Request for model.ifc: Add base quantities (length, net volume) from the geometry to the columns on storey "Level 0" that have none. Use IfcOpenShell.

First a look at what the model holds.

```python
import ifcopenshell
import ifcopenshell.util.element
import ifcopenshell.util.unit

model = ifcopenshell.open("model.ifc")
print(model.schema)
for unit_type in ("LENGTHUNIT", "AREAUNIT", "VOLUMEUNIT"):
    print(unit_type, ifcopenshell.util.unit.calculate_unit_scale(model, unit_type))
storey = next(s for s in model.by_type("IfcBuildingStorey") if s.Name == "Level 0")
columns = [e for e in ifcopenshell.util.element.get_decomposition(storey) if e.is_a("IfcColumn")]
for e in sorted(columns, key=lambda e: e.id()):
    print(e.id(), e.is_a(), e.Name, list(ifcopenshell.util.element.get_psets(e, qtos_only=True)), sep=" | ")
```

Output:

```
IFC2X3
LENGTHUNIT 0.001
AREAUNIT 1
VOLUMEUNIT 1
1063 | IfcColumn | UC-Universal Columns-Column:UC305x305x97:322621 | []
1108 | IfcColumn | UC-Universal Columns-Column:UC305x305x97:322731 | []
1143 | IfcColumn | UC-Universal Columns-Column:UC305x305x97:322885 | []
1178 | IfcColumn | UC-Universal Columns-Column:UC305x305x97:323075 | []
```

```python
import ifcopenshell
import ifcopenshell.api.pset
import ifcopenshell.geom
import ifcopenshell.util.element
import ifcopenshell.util.shape
import ifcopenshell.util.unit

model = ifcopenshell.open("model.ifc")
unit_scale = ifcopenshell.util.unit.calculate_unit_scale(model)
volume_scale = ifcopenshell.util.unit.calculate_unit_scale(model, "VOLUMEUNIT")
settings = ifcopenshell.geom.settings()

storey = next(s for s in model.by_type("IfcBuildingStorey") if s.Name == "Level 0")
columns = [e for e in ifcopenshell.util.element.get_decomposition(storey) if e.is_a("IfcColumn")]

for e in sorted(columns, key=lambda e: e.id()):
    if ifcopenshell.util.element.get_psets(e, qtos_only=True, should_inherit=False):
        continue
    # Geometry comes back in metres, in the element's own axes.
    shape = ifcopenshell.geom.create_shape(settings, e)
    values = {
        "Length": ifcopenshell.util.shape.get_z(shape.geometry) / unit_scale,
        "NetVolume": ifcopenshell.util.shape.get_volume(shape.geometry) / volume_scale,
    }
    qto = ifcopenshell.api.pset.add_qto(model, product=e, name="BaseQuantities")
    ifcopenshell.api.pset.edit_qto(model, qto=qto, properties=values)
    print(e.id(), {k: round(v, 3) for k, v in values.items()})

model.write("model_edited.ifc")
```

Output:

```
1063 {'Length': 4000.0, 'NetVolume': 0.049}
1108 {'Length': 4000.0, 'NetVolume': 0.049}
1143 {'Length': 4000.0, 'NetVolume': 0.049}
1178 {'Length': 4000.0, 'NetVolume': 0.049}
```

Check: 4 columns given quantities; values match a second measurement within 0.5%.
